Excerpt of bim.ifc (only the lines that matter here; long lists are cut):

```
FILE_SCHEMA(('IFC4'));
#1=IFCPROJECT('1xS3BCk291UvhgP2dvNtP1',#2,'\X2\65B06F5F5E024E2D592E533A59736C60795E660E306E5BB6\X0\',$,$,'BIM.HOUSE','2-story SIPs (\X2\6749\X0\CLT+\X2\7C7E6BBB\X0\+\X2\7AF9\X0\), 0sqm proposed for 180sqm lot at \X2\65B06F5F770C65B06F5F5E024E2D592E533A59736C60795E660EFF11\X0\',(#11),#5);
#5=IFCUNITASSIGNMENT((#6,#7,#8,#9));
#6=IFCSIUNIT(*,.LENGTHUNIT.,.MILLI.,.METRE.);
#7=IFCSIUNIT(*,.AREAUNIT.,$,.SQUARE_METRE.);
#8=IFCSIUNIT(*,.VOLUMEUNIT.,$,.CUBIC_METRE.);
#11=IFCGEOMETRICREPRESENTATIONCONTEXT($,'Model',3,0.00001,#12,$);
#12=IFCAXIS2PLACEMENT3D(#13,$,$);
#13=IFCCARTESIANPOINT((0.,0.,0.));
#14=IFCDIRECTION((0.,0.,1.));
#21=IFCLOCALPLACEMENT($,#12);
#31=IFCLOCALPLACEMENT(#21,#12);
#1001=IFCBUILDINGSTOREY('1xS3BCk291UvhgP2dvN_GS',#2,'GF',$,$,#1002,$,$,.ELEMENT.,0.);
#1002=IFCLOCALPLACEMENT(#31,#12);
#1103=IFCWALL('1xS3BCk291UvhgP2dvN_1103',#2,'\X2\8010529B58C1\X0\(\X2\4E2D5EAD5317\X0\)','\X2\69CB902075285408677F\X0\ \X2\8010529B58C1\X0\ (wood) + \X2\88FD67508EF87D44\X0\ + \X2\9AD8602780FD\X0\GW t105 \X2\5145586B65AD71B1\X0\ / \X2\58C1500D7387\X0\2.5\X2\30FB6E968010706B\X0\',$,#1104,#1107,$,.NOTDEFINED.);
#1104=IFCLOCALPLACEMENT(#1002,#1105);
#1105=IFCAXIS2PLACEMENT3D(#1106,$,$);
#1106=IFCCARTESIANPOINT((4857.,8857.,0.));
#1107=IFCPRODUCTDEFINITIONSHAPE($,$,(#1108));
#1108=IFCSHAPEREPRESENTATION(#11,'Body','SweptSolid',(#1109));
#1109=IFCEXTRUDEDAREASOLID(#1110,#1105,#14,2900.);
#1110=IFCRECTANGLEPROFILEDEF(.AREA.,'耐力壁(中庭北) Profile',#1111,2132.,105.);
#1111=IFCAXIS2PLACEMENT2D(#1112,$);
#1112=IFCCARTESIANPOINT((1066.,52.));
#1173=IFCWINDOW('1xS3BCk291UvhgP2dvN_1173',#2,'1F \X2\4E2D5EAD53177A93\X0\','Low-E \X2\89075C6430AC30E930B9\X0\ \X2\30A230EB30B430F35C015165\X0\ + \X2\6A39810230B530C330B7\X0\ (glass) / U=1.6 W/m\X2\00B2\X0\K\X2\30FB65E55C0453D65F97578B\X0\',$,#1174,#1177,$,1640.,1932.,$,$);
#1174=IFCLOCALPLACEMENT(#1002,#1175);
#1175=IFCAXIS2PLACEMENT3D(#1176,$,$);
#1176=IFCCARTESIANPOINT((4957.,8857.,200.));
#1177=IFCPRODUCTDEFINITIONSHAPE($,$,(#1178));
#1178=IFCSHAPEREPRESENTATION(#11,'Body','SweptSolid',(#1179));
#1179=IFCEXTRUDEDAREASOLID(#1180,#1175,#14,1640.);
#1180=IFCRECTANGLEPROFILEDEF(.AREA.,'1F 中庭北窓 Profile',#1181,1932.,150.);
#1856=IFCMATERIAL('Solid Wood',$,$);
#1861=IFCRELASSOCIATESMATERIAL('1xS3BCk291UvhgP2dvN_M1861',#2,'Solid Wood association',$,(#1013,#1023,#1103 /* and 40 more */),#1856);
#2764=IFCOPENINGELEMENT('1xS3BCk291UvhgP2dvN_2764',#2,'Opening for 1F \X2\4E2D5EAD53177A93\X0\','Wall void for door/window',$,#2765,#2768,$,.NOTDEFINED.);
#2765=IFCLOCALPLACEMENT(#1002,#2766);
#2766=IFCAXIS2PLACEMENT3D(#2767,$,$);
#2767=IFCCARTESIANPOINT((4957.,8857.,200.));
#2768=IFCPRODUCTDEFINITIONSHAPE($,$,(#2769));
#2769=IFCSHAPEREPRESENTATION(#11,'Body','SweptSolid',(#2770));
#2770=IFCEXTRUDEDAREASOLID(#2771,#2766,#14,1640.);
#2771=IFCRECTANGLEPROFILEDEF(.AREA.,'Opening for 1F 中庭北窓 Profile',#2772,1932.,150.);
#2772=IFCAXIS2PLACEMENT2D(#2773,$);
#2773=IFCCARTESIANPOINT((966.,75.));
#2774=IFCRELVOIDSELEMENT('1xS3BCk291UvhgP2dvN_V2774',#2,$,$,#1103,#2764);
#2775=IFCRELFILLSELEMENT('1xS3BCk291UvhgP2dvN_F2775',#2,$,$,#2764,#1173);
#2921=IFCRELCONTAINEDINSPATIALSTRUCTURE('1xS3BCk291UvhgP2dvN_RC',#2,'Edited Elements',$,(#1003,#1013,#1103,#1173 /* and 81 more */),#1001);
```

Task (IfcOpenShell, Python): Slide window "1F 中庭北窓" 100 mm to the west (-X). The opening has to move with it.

```python
import ifcopenshell
import ifcopenshell.api.geometry
import ifcopenshell.util.placement

model = ifcopenshell.open("bim.ifc")

window = model.by_guid("1xS3BCk291UvhgP2dvN_1173")
opening = window.FillsVoids[0].RelatingOpeningElement
wall = opening.VoidsElements[0].RelatingBuildingElement

wall_matrix = ifcopenshell.util.placement.get_local_placement(wall.ObjectPlacement)
shift = wall_matrix[:3, 0] * -100.0
before = ifcopenshell.util.placement.get_local_placement(window.ObjectPlacement)[:3, 3].copy()

# The window is not placed relative to its opening, so move both.
for product in (opening, window):
    matrix = ifcopenshell.util.placement.get_local_placement(product.ObjectPlacement)
    matrix[:3, 3] += shift
    ifcopenshell.api.geometry.edit_object_placement(model, product=product, matrix=matrix, is_si=False)

after = ifcopenshell.util.placement.get_local_placement(window.ObjectPlacement)[:3, 3]
print("window moved by", (after - before).round(3) + 0.0)

model.write("bim-out.ifc")
```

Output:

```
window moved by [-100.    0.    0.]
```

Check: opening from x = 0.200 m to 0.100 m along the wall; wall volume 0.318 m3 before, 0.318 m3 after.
